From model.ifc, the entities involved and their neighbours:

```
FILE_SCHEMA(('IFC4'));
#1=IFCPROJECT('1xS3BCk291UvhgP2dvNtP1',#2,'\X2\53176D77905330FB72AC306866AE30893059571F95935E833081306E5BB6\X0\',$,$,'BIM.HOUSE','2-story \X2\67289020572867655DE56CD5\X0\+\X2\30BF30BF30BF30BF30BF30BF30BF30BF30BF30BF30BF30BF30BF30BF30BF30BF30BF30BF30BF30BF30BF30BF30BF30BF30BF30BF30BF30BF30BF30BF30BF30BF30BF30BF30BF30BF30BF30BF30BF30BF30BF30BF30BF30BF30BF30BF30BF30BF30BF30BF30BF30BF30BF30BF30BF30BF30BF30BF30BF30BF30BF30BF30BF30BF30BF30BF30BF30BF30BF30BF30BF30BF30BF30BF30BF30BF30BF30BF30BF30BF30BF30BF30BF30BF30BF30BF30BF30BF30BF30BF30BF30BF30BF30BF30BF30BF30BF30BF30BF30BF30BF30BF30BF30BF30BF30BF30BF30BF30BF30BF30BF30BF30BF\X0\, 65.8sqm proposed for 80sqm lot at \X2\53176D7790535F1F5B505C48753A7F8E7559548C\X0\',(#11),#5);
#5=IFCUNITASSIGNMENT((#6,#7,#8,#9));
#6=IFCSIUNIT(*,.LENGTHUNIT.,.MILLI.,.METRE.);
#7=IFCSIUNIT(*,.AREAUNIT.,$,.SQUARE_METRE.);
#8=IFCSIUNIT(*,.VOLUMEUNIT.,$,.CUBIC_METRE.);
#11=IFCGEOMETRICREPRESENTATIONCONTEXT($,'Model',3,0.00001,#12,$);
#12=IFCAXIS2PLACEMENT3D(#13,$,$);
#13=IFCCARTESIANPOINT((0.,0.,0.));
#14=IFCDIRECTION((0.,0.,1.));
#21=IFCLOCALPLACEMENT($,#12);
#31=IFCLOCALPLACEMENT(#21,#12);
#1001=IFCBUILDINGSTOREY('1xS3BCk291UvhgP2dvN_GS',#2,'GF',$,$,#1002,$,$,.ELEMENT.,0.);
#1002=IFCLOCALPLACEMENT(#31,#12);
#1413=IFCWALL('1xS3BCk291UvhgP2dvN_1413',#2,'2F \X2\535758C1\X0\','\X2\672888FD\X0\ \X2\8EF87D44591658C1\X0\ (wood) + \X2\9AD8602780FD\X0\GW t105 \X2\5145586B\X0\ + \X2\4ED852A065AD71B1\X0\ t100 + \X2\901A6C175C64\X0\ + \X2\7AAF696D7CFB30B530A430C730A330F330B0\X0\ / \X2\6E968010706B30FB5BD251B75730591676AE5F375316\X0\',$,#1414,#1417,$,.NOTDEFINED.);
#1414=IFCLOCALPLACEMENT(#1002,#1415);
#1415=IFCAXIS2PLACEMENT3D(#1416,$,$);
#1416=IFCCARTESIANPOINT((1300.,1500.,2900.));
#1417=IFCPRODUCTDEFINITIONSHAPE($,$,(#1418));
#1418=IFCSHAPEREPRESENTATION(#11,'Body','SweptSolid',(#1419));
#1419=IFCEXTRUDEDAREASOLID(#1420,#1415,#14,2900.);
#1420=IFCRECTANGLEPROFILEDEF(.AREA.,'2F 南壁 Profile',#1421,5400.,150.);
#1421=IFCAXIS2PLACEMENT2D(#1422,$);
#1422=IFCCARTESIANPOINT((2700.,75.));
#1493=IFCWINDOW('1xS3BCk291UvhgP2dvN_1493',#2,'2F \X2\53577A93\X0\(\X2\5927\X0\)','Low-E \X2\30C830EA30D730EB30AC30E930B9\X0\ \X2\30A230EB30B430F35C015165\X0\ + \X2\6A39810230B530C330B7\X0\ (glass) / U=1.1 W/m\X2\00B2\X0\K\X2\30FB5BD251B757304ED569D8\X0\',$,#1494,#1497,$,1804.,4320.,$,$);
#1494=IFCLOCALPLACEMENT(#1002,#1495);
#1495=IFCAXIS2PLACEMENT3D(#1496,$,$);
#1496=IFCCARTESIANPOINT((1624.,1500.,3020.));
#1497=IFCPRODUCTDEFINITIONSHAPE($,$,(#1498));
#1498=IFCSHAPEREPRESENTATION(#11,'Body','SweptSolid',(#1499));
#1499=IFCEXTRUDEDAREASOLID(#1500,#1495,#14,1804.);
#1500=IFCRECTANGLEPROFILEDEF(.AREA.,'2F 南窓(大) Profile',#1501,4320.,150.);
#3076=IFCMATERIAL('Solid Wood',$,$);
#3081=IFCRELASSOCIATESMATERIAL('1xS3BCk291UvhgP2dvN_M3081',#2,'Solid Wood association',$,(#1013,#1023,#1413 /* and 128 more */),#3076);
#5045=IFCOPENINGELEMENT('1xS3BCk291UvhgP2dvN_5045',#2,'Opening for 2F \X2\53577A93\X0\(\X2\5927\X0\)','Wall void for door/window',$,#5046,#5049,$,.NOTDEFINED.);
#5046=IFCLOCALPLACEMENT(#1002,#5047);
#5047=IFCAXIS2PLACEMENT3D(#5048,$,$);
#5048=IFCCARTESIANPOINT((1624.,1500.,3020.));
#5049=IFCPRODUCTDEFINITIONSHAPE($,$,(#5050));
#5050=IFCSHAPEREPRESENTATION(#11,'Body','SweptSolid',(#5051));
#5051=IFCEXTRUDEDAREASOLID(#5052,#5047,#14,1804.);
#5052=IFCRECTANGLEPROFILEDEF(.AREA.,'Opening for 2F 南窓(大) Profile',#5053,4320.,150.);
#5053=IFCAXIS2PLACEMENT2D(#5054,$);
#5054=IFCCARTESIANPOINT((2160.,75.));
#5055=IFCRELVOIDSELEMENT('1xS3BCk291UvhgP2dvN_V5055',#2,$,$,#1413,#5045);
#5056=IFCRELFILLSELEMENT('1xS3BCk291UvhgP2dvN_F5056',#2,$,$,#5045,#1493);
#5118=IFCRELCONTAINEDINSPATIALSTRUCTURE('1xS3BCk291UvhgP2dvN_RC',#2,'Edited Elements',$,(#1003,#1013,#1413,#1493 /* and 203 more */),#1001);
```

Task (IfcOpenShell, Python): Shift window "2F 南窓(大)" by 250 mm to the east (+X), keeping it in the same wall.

```python
import ifcopenshell
import ifcopenshell.api.geometry
import ifcopenshell.util.placement
import ifcopenshell.util.unit

model = ifcopenshell.open("model.ifc")
unit_scale = ifcopenshell.util.unit.calculate_unit_scale(model)

window = model.by_guid("1xS3BCk291UvhgP2dvN_1493")
opening = window.FillsVoids[0].RelatingOpeningElement
wall = opening.VoidsElements[0].RelatingBuildingElement

wall_matrix = ifcopenshell.util.placement.get_local_placement(wall.ObjectPlacement)
shift = wall_matrix[:3, 0] * 0.25 / unit_scale
before = ifcopenshell.util.placement.get_local_placement(window.ObjectPlacement)[:3, 3].copy()

# The window is not placed relative to its opening, so move both.
for product in (opening, window):
    matrix = ifcopenshell.util.placement.get_local_placement(product.ObjectPlacement)
    matrix[:3, 3] += shift
    ifcopenshell.api.geometry.edit_object_placement(model, product=product, matrix=matrix, is_si=False)

after = ifcopenshell.util.placement.get_local_placement(window.ObjectPlacement)[:3, 3]
print("window moved by", (after - before).round(3) + 0.0)

model.write("model_edited.ifc")
```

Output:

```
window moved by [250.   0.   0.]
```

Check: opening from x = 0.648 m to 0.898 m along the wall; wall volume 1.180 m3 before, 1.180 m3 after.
